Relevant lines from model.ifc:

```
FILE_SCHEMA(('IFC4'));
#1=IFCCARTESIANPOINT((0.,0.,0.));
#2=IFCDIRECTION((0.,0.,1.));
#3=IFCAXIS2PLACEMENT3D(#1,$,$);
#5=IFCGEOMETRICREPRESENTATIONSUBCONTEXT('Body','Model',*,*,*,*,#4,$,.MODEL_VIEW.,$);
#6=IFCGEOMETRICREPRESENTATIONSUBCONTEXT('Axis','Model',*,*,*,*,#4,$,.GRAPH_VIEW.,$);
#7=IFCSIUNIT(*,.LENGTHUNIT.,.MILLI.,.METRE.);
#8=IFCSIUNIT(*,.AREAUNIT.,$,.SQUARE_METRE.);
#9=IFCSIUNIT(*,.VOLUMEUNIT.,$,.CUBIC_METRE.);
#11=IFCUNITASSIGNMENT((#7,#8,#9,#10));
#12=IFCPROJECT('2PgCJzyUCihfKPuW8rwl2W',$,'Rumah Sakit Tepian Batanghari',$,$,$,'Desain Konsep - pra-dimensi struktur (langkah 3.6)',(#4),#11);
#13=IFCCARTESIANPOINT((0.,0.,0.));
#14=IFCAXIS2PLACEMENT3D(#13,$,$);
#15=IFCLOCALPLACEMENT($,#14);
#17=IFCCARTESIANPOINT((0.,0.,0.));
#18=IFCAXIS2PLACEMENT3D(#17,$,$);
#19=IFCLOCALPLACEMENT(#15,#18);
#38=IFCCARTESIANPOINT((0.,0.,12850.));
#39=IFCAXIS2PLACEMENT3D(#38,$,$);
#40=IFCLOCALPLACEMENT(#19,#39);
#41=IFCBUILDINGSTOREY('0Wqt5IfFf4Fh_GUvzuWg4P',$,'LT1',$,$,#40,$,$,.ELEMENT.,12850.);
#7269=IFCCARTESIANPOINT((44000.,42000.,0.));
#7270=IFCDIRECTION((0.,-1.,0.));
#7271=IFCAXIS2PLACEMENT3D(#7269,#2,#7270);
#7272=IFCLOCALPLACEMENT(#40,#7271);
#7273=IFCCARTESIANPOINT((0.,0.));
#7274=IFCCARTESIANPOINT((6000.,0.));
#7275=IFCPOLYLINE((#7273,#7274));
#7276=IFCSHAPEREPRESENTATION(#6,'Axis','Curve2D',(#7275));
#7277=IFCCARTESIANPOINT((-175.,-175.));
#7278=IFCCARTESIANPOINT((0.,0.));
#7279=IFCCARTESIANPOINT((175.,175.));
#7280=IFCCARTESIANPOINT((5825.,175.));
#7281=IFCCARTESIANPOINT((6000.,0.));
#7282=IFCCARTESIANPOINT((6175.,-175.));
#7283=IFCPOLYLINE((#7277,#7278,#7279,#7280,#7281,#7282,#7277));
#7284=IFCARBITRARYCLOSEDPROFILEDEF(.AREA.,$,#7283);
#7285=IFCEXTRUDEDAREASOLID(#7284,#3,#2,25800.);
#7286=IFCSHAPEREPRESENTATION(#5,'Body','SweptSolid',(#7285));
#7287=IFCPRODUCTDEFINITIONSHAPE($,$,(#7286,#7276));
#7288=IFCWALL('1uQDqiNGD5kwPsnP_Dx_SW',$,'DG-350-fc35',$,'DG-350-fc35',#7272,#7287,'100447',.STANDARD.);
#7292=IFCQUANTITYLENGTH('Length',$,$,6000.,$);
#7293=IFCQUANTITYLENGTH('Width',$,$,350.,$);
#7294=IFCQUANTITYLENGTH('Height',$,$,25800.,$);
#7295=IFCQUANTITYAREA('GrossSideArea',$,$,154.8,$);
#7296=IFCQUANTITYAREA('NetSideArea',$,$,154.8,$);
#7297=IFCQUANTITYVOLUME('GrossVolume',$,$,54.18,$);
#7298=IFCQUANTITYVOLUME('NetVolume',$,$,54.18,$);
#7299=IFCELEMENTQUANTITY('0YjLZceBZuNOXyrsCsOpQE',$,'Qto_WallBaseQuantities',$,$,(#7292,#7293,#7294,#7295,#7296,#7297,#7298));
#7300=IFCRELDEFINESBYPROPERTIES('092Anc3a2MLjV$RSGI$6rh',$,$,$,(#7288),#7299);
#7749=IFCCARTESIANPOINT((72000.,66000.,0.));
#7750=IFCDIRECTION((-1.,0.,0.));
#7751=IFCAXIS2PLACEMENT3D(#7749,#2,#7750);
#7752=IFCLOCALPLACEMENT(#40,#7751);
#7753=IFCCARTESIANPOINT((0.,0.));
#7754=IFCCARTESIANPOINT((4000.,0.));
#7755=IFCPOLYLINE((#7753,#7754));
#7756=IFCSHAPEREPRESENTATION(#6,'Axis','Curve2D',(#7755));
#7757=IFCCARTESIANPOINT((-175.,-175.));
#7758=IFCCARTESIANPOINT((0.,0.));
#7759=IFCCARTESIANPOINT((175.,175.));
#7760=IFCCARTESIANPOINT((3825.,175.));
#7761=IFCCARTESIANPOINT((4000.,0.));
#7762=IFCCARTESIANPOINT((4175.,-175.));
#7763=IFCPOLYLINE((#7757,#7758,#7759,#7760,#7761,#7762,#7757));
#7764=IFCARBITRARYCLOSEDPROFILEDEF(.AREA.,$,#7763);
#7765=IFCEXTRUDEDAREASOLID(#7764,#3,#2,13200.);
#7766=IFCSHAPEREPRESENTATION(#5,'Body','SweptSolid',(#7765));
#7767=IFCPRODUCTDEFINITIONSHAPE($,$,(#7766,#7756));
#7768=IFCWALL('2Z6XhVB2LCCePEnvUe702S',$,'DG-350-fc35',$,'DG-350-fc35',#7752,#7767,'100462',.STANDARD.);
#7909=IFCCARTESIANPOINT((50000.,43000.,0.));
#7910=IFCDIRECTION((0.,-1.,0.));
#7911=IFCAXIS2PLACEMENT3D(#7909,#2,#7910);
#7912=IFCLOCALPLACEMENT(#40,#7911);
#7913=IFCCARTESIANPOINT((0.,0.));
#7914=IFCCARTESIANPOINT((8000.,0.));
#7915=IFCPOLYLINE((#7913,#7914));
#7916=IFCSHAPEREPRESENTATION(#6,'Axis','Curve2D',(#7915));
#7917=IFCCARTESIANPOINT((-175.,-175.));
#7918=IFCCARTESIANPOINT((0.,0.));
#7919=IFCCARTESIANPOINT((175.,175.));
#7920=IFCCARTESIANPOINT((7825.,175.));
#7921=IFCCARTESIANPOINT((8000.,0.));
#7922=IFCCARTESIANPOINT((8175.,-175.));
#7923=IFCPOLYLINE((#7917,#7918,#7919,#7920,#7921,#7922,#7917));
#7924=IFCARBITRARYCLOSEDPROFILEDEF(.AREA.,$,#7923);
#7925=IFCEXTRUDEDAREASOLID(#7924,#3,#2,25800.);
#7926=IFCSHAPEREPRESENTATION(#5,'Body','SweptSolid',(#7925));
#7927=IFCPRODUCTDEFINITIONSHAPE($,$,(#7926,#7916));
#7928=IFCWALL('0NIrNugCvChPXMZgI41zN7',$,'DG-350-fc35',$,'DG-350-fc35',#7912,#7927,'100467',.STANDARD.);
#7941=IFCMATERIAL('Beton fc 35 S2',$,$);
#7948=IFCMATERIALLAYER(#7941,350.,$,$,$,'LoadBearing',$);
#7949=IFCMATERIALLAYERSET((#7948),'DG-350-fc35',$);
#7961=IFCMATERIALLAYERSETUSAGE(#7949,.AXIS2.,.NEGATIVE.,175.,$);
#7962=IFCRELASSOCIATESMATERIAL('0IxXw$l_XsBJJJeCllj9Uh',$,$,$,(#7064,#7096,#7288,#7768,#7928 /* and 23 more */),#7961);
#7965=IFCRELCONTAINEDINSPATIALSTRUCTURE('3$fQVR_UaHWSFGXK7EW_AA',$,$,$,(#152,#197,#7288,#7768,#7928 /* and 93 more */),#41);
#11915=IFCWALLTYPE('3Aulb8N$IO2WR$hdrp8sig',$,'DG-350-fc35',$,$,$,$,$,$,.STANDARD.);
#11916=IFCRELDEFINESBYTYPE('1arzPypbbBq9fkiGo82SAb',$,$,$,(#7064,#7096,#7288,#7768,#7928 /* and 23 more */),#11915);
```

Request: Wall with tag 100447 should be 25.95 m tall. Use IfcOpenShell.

```python
import ifcopenshell
import ifcopenshell.api.pset
import ifcopenshell.geom
import ifcopenshell.util.element
import ifcopenshell.util.representation
import ifcopenshell.util.shape
import ifcopenshell.util.unit

model = ifcopenshell.open("model.ifc")
unit_scale = ifcopenshell.util.unit.calculate_unit_scale(model)
area_scale = ifcopenshell.util.unit.calculate_unit_scale(model, "AREAUNIT")
volume_scale = ifcopenshell.util.unit.calculate_unit_scale(model, "VOLUMEUNIT")
settings = ifcopenshell.geom.settings()


def volume(element):
    """Net volume in cubic metres, openings subtracted."""
    shape = ifcopenshell.geom.create_shape(settings, element)
    return ifcopenshell.util.shape.get_volume(shape.geometry)


wall = model.by_guid("1uQDqiNGD5kwPsnP_Dx_SW")
before = volume(wall)

body = ifcopenshell.util.representation.get_representation(wall, "Model", "Body")
solid = body.Items[0]
old_height = solid.Depth
solid.Depth = 25.95 / unit_scale
after = volume(wall)
thickness = 0.35  # wall thickness in metres

# Update the stored height, areas and volumes.
qto = model.by_id(ifcopenshell.util.element.get_pset(wall, "Qto_WallBaseQuantities", should_inherit=False)["id"])
ifcopenshell.api.pset.edit_qto(model, qto=qto, properties={
    "Height": solid.Depth,
    "GrossSideArea": ifcopenshell.util.element.get_pset(wall, "Qto_WallBaseQuantities", "GrossSideArea") * solid.Depth / old_height,
    "NetSideArea": after / thickness / area_scale,
    "GrossVolume": ifcopenshell.util.element.get_pset(wall, "Qto_WallBaseQuantities", "GrossVolume") * solid.Depth / old_height,
    "NetVolume": after / volume_scale,
})

print(f"height {old_height:g} -> {solid.Depth:g}, volume {before:.3f} -> {after:.3f} m3")

model.write("model_edited.ifc")
```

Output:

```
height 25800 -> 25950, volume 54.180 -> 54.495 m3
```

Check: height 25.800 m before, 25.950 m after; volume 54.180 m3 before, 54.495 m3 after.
